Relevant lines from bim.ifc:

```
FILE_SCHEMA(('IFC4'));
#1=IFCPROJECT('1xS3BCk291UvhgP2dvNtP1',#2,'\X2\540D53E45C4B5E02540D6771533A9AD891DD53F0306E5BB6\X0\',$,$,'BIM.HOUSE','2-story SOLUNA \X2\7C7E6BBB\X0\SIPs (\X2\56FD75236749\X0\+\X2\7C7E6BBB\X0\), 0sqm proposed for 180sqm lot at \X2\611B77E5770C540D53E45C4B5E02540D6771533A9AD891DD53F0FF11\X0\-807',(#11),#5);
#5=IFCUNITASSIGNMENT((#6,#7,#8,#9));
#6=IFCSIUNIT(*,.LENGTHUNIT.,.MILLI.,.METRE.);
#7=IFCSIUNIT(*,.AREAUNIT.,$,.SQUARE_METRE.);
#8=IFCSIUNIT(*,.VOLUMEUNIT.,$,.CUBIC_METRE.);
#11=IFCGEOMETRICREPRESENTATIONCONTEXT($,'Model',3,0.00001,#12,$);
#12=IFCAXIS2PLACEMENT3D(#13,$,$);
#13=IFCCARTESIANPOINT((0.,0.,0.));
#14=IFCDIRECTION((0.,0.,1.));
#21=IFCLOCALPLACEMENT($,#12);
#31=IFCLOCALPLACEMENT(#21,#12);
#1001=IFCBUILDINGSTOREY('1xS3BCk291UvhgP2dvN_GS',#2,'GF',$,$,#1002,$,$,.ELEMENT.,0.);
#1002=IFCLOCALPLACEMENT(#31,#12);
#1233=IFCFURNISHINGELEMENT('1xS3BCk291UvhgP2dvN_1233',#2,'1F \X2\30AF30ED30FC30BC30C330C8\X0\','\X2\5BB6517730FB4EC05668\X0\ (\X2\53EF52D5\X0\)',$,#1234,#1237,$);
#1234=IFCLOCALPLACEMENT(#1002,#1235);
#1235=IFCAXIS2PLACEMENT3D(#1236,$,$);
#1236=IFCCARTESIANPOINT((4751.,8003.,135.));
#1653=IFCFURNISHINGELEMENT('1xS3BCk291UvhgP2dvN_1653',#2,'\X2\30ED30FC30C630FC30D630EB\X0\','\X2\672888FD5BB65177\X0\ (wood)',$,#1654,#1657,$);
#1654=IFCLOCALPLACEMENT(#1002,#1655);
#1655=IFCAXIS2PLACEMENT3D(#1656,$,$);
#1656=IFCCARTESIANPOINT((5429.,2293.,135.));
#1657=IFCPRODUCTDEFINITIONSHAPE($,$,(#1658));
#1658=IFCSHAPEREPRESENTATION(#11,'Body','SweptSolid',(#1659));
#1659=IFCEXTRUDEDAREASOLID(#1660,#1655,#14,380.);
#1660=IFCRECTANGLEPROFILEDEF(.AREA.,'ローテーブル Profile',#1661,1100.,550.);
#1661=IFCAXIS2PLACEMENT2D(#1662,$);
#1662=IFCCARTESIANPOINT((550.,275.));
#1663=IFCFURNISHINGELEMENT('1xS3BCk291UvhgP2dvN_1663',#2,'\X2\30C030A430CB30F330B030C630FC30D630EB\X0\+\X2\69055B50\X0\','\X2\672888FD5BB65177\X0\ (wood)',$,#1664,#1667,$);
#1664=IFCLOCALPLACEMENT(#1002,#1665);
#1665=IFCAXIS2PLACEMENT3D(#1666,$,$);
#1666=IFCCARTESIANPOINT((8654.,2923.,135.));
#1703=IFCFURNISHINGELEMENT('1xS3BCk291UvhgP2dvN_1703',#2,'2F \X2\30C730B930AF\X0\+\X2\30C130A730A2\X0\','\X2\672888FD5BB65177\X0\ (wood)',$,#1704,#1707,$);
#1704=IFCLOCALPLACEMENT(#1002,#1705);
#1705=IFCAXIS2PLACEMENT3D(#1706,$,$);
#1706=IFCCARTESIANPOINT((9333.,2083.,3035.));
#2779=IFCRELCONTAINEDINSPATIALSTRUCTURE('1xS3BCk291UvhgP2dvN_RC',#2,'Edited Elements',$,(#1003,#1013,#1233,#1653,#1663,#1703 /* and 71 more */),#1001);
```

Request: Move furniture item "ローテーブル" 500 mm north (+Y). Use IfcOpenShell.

```python
import ifcopenshell
import ifcopenshell.api.geometry
import ifcopenshell.util.placement
import ifcopenshell.util.unit

model = ifcopenshell.open("bim.ifc")
unit_scale = ifcopenshell.util.unit.calculate_unit_scale(model)

item = model.by_guid("1xS3BCk291UvhgP2dvN_1653")
matrix = ifcopenshell.util.placement.get_local_placement(item.ObjectPlacement)
matrix[1, 3] += 0.5 / unit_scale
ifcopenshell.api.geometry.edit_object_placement(model, product=item, matrix=matrix, is_si=False)

print(ifcopenshell.util.placement.get_local_placement(item.ObjectPlacement).round(3) + 0.0)

model.write("bim_updated.ifc")
```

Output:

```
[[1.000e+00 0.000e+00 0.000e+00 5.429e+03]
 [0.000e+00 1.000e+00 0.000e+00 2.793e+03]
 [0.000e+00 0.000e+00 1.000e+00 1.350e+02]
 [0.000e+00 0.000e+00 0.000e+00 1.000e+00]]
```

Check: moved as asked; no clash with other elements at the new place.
